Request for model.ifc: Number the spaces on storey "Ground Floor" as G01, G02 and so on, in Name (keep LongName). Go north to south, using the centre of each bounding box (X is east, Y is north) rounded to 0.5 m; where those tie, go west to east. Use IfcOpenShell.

First a look at what the model holds.

```python
import ifcopenshell
import ifcopenshell.util.element
import ifcopenshell.util.placement

model = ifcopenshell.open("model.ifc")
print(model.schema)
storey = next(s for s in model.by_type("IfcBuildingStorey") if s.Name == "Ground Floor")
spaces = [e for e in ifcopenshell.util.element.get_decomposition(storey) if e.is_a("IfcSpace")]
for e in sorted(spaces, key=lambda e: e.id()):
    origin = ifcopenshell.util.placement.get_local_placement(e.ObjectPlacement)[:3, 3]
    print(e.id(), e.Name, e.LongName, origin.round(2) + 0.0, sep=" | ")
```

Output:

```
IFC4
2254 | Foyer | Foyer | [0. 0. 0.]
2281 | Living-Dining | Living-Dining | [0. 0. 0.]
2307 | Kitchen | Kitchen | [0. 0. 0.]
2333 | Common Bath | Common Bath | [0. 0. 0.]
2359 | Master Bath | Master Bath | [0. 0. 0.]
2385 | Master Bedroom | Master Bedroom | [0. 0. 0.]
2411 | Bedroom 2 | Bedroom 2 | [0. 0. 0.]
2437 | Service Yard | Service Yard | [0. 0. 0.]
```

```python
import ifcopenshell
import ifcopenshell.geom
import ifcopenshell.util.element
import ifcopenshell.util.shape

model = ifcopenshell.open("model.ifc")
settings = ifcopenshell.geom.settings()
settings.set("use-world-coords", True)


def centre(element):
    shape = ifcopenshell.geom.create_shape(settings, element)
    return ifcopenshell.util.shape.get_bbox_centroid(shape.geometry)


storey = next(s for s in model.by_type("IfcBuildingStorey") if s.Name == "Ground Floor")
spaces = [e for e in ifcopenshell.util.element.get_decomposition(storey) if e.is_a("IfcSpace")]

# Insertion points can sit at a corner or the storey origin, so sort by the geometry (in metres).
centres = {e: centre(e) for e in spaces}
spaces.sort(key=lambda e: (-round(centres[e][1] / 0.5), centres[e][0]))

for i, e in enumerate(spaces, start=1):
    number = f"G{i:02d}"
    e.Name = number
    print(e.id(), number)

model.write("model_rev.ifc")
```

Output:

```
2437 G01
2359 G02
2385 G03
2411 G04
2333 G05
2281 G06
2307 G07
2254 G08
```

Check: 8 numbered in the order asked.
